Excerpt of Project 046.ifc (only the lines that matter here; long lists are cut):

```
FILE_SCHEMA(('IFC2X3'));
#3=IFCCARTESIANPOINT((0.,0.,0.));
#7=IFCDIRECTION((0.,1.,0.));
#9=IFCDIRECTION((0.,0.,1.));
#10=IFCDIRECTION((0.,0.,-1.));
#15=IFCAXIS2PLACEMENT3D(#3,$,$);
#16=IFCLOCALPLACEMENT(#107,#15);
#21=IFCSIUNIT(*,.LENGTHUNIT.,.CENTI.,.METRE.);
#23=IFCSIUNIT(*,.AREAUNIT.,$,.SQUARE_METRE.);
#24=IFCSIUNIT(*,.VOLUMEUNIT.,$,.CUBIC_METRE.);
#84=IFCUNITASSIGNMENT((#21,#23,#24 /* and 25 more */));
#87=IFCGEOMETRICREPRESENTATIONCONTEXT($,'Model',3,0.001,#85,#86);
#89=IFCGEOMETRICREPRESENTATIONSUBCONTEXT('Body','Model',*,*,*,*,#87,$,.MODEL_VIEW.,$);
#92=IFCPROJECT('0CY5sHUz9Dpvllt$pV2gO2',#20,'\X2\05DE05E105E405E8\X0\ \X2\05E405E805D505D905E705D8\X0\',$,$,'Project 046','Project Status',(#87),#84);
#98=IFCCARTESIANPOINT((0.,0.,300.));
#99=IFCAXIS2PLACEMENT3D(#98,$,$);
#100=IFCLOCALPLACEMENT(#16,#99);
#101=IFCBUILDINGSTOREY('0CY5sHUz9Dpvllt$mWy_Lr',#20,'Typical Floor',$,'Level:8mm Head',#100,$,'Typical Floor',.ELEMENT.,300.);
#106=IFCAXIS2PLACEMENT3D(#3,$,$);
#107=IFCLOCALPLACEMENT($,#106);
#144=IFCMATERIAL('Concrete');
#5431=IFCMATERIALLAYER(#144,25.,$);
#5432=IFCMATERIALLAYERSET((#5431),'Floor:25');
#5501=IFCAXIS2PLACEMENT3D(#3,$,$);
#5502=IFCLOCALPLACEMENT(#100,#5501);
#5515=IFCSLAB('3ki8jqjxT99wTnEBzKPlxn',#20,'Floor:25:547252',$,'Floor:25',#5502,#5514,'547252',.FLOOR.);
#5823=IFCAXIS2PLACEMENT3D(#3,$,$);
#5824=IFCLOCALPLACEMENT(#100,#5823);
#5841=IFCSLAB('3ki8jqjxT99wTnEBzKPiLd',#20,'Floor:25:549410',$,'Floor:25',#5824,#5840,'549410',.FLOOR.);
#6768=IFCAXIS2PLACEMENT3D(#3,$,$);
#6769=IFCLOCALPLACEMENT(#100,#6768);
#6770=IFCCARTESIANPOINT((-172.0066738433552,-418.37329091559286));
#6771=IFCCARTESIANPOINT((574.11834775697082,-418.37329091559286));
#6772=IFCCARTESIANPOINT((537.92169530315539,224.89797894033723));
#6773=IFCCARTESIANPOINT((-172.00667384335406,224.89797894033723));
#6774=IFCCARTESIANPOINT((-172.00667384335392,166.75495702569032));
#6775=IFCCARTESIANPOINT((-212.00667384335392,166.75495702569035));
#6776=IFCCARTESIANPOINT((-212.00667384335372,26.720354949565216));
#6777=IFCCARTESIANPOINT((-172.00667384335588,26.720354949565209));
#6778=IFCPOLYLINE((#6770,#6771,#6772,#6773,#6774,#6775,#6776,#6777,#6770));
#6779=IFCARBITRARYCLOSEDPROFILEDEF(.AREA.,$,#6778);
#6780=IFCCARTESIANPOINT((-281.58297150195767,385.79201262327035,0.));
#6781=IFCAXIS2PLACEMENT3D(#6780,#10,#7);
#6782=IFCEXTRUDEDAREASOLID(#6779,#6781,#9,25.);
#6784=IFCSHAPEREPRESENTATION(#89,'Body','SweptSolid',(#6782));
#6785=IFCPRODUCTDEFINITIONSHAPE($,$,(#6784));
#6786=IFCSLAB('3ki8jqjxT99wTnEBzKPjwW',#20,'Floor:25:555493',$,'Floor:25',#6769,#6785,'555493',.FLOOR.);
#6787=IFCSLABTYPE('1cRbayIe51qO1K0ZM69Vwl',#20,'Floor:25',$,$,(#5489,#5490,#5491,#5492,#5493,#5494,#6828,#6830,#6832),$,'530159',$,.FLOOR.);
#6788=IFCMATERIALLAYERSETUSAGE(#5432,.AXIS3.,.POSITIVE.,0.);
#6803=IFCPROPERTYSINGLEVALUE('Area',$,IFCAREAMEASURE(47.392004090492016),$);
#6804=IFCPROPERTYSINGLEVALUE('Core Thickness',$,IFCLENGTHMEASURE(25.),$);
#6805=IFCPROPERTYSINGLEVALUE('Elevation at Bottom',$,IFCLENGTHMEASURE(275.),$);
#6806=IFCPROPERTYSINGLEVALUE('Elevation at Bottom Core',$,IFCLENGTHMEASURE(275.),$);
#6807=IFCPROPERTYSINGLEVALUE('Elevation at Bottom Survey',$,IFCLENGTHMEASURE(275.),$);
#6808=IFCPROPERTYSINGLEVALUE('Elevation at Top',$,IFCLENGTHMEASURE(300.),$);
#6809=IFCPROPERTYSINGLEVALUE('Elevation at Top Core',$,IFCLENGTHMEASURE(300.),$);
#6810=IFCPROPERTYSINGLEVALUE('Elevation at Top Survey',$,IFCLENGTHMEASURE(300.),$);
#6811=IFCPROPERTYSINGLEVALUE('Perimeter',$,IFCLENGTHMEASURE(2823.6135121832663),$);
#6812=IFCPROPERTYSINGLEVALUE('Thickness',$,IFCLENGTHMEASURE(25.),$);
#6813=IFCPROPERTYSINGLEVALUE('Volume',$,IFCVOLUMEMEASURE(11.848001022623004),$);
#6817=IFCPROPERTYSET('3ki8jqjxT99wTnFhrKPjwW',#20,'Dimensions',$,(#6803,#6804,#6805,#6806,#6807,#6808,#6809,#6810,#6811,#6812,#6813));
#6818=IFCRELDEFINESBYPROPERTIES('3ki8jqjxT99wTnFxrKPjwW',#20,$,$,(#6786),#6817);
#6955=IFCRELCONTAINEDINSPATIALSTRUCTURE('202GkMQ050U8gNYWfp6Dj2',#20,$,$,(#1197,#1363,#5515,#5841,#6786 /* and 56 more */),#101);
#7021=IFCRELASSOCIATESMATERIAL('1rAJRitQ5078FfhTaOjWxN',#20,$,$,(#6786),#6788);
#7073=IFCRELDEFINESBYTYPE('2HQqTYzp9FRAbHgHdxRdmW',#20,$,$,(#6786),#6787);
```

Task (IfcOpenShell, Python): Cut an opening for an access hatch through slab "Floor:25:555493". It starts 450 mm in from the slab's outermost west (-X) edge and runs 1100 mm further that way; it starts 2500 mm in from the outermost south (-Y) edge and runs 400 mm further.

```python
import numpy as np
import ifcopenshell
import ifcopenshell.api.feature
import ifcopenshell.api.geometry
import ifcopenshell.api.pset
import ifcopenshell.api.root
import ifcopenshell.geom
import ifcopenshell.util.element
import ifcopenshell.util.placement
import ifcopenshell.util.representation
import ifcopenshell.util.shape
import ifcopenshell.util.unit

model = ifcopenshell.open("Project 046.ifc")
unit_scale = ifcopenshell.util.unit.calculate_unit_scale(model)
area_scale = ifcopenshell.util.unit.calculate_unit_scale(model, "AREAUNIT")
volume_scale = ifcopenshell.util.unit.calculate_unit_scale(model, "VOLUMEUNIT")
settings = ifcopenshell.geom.settings()


def volume(element):
    """Net volume in cubic metres, openings subtracted."""
    shape = ifcopenshell.geom.create_shape(settings, element)
    return ifcopenshell.util.shape.get_volume(shape.geometry)


slab = model.by_guid("3ki8jqjxT99wTnEBzKPjwW")
before = volume(slab)

# Extent in the slab's own axes, in metres. The edges named are its -X and -Y sides.
slab_shape = ifcopenshell.geom.create_shape(settings, slab)
vertices = ifcopenshell.util.shape.get_vertices(slab_shape.geometry)
x_min, y_min, bottom = vertices.min(axis=0)
top = vertices[:, 2].max()

opening = ifcopenshell.api.root.create_entity(model, ifc_class="IfcOpeningElement", name="Access hatch opening")
context = ifcopenshell.util.representation.get_context(model, "Model", "Body", "MODEL_VIEW")
width, depth = 1.1, 0.4
outline = [(0.0, 0.0), (width, 0.0), (width, depth), (0.0, depth), (0.0, 0.0)]
# Overshoot both faces by 50 mm so the cut is clean.
shape = ifcopenshell.api.geometry.add_slab_representation(
    model, context=context, depth=top - bottom + 0.1, polyline=outline
)
ifcopenshell.api.geometry.assign_representation(model, product=opening, representation=shape)

matrix = ifcopenshell.util.placement.get_local_placement(slab.ObjectPlacement)
matrix[:, 3] = matrix @ np.append(np.array([x_min + 0.45, y_min + 2.5, bottom - 0.05]) / unit_scale, 1.0)
ifcopenshell.api.geometry.edit_object_placement(model, product=opening, matrix=matrix, is_si=False)
ifcopenshell.api.feature.add_feature(model, feature=opening, element=slab)

after = volume(slab)

# Update the slab's stored quantities.
pset = model.by_id(ifcopenshell.util.element.get_pset(slab, "Dimensions", should_inherit=False)["id"])
ifcopenshell.api.pset.edit_pset(model, pset=pset, properties={
    "Area": model.create_entity("IfcAreaMeasure", after / (top - bottom) / area_scale),
    "Volume": model.create_entity("IfcVolumeMeasure", after / volume_scale),
})

print(f"slab volume {before:.3f} -> {after:.3f} m3")

model.write("Project 046_updated.ifc")
```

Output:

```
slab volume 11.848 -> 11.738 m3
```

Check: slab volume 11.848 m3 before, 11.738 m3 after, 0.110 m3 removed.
